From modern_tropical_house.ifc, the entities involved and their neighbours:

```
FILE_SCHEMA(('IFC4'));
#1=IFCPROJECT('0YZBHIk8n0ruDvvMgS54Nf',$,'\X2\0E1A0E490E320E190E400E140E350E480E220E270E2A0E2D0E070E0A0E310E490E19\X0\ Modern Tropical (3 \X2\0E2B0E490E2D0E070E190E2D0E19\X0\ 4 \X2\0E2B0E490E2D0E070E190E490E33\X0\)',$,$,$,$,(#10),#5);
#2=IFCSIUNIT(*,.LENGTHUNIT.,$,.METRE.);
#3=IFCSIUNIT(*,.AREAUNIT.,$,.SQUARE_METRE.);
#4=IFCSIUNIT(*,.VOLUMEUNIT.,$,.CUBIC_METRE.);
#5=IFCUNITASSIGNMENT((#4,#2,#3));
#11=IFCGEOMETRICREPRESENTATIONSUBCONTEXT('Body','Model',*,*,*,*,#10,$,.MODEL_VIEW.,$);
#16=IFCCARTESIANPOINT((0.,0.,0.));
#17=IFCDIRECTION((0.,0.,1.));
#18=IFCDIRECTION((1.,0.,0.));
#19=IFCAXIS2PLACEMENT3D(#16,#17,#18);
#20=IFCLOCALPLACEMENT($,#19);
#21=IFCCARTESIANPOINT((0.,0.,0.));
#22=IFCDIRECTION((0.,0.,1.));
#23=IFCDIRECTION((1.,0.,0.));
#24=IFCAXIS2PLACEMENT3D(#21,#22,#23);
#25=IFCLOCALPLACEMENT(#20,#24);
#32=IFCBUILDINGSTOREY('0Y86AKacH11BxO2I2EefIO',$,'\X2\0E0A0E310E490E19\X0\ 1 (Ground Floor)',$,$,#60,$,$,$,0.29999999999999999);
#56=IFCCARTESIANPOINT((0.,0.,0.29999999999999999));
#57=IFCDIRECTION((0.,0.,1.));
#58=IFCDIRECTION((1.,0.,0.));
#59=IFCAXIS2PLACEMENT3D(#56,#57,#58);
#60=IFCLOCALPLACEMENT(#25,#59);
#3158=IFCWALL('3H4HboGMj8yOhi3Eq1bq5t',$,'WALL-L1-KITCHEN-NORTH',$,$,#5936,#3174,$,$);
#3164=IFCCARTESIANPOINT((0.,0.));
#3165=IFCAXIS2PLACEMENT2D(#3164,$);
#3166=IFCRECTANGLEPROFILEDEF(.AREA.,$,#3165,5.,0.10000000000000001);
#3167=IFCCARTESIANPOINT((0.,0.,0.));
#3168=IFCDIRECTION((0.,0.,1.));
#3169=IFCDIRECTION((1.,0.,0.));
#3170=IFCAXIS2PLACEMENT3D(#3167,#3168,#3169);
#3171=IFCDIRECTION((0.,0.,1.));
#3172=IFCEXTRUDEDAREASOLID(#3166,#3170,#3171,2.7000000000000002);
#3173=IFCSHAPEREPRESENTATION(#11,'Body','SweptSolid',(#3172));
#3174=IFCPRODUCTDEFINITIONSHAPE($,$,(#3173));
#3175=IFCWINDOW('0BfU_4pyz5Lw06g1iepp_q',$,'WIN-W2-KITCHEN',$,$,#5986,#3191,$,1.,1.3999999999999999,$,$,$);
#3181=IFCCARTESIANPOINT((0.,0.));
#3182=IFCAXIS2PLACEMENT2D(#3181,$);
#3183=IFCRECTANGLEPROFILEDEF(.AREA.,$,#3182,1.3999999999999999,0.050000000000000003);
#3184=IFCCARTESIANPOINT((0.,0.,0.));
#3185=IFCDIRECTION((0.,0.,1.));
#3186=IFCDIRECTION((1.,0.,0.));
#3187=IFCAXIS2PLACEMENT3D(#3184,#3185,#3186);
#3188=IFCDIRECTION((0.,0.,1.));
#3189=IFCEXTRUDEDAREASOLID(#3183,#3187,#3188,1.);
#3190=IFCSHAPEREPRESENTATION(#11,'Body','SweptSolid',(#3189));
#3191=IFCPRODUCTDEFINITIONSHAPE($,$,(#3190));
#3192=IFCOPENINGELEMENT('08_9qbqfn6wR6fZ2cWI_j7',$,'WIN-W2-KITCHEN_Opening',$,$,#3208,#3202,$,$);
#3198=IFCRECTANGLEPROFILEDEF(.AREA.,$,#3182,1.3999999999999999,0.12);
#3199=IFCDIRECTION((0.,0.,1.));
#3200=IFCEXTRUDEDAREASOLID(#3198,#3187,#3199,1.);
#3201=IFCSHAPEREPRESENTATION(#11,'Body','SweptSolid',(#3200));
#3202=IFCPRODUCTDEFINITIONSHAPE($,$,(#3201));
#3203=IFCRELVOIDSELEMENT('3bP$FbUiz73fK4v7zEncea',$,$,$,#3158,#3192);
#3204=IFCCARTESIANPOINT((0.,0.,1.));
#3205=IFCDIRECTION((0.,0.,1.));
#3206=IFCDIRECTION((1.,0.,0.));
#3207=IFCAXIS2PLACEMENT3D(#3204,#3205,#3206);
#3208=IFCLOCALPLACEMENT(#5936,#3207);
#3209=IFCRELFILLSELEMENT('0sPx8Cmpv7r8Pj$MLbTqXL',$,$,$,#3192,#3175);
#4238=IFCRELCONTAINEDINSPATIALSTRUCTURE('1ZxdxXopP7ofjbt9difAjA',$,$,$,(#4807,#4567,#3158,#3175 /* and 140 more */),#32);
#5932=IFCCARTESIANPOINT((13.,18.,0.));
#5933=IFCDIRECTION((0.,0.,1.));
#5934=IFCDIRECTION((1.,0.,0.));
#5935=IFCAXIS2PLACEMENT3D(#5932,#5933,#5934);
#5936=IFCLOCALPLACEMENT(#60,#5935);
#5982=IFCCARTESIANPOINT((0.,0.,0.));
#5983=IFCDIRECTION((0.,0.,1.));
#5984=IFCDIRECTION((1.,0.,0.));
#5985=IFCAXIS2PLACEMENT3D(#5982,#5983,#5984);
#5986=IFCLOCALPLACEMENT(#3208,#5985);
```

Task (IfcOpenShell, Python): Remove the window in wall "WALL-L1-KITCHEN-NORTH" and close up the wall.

```python
import ifcopenshell
import ifcopenshell.api.feature
import ifcopenshell.api.root
import ifcopenshell.geom
import ifcopenshell.util.shape

model = ifcopenshell.open("modern_tropical_house.ifc")
settings = ifcopenshell.geom.settings()


def volume(element):
    """Net volume in cubic metres, openings subtracted."""
    shape = ifcopenshell.geom.create_shape(settings, element)
    return ifcopenshell.util.shape.get_volume(shape.geometry)


window = model.by_guid("0BfU_4pyz5Lw06g1iepp_q")
opening = window.FillsVoids[0].RelatingOpeningElement
wall = opening.VoidsElements[0].RelatingBuildingElement
before = volume(wall)

ifcopenshell.api.root.remove_product(model, product=window)
ifcopenshell.api.feature.remove_feature(model, feature=opening)

after = volume(wall)

print(f"wall volume {before:.3f} -> {after:.3f} m3")

model.write("modern_tropical_house_rev.ifc")
```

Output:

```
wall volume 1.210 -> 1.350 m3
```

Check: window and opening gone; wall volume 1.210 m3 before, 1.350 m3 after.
